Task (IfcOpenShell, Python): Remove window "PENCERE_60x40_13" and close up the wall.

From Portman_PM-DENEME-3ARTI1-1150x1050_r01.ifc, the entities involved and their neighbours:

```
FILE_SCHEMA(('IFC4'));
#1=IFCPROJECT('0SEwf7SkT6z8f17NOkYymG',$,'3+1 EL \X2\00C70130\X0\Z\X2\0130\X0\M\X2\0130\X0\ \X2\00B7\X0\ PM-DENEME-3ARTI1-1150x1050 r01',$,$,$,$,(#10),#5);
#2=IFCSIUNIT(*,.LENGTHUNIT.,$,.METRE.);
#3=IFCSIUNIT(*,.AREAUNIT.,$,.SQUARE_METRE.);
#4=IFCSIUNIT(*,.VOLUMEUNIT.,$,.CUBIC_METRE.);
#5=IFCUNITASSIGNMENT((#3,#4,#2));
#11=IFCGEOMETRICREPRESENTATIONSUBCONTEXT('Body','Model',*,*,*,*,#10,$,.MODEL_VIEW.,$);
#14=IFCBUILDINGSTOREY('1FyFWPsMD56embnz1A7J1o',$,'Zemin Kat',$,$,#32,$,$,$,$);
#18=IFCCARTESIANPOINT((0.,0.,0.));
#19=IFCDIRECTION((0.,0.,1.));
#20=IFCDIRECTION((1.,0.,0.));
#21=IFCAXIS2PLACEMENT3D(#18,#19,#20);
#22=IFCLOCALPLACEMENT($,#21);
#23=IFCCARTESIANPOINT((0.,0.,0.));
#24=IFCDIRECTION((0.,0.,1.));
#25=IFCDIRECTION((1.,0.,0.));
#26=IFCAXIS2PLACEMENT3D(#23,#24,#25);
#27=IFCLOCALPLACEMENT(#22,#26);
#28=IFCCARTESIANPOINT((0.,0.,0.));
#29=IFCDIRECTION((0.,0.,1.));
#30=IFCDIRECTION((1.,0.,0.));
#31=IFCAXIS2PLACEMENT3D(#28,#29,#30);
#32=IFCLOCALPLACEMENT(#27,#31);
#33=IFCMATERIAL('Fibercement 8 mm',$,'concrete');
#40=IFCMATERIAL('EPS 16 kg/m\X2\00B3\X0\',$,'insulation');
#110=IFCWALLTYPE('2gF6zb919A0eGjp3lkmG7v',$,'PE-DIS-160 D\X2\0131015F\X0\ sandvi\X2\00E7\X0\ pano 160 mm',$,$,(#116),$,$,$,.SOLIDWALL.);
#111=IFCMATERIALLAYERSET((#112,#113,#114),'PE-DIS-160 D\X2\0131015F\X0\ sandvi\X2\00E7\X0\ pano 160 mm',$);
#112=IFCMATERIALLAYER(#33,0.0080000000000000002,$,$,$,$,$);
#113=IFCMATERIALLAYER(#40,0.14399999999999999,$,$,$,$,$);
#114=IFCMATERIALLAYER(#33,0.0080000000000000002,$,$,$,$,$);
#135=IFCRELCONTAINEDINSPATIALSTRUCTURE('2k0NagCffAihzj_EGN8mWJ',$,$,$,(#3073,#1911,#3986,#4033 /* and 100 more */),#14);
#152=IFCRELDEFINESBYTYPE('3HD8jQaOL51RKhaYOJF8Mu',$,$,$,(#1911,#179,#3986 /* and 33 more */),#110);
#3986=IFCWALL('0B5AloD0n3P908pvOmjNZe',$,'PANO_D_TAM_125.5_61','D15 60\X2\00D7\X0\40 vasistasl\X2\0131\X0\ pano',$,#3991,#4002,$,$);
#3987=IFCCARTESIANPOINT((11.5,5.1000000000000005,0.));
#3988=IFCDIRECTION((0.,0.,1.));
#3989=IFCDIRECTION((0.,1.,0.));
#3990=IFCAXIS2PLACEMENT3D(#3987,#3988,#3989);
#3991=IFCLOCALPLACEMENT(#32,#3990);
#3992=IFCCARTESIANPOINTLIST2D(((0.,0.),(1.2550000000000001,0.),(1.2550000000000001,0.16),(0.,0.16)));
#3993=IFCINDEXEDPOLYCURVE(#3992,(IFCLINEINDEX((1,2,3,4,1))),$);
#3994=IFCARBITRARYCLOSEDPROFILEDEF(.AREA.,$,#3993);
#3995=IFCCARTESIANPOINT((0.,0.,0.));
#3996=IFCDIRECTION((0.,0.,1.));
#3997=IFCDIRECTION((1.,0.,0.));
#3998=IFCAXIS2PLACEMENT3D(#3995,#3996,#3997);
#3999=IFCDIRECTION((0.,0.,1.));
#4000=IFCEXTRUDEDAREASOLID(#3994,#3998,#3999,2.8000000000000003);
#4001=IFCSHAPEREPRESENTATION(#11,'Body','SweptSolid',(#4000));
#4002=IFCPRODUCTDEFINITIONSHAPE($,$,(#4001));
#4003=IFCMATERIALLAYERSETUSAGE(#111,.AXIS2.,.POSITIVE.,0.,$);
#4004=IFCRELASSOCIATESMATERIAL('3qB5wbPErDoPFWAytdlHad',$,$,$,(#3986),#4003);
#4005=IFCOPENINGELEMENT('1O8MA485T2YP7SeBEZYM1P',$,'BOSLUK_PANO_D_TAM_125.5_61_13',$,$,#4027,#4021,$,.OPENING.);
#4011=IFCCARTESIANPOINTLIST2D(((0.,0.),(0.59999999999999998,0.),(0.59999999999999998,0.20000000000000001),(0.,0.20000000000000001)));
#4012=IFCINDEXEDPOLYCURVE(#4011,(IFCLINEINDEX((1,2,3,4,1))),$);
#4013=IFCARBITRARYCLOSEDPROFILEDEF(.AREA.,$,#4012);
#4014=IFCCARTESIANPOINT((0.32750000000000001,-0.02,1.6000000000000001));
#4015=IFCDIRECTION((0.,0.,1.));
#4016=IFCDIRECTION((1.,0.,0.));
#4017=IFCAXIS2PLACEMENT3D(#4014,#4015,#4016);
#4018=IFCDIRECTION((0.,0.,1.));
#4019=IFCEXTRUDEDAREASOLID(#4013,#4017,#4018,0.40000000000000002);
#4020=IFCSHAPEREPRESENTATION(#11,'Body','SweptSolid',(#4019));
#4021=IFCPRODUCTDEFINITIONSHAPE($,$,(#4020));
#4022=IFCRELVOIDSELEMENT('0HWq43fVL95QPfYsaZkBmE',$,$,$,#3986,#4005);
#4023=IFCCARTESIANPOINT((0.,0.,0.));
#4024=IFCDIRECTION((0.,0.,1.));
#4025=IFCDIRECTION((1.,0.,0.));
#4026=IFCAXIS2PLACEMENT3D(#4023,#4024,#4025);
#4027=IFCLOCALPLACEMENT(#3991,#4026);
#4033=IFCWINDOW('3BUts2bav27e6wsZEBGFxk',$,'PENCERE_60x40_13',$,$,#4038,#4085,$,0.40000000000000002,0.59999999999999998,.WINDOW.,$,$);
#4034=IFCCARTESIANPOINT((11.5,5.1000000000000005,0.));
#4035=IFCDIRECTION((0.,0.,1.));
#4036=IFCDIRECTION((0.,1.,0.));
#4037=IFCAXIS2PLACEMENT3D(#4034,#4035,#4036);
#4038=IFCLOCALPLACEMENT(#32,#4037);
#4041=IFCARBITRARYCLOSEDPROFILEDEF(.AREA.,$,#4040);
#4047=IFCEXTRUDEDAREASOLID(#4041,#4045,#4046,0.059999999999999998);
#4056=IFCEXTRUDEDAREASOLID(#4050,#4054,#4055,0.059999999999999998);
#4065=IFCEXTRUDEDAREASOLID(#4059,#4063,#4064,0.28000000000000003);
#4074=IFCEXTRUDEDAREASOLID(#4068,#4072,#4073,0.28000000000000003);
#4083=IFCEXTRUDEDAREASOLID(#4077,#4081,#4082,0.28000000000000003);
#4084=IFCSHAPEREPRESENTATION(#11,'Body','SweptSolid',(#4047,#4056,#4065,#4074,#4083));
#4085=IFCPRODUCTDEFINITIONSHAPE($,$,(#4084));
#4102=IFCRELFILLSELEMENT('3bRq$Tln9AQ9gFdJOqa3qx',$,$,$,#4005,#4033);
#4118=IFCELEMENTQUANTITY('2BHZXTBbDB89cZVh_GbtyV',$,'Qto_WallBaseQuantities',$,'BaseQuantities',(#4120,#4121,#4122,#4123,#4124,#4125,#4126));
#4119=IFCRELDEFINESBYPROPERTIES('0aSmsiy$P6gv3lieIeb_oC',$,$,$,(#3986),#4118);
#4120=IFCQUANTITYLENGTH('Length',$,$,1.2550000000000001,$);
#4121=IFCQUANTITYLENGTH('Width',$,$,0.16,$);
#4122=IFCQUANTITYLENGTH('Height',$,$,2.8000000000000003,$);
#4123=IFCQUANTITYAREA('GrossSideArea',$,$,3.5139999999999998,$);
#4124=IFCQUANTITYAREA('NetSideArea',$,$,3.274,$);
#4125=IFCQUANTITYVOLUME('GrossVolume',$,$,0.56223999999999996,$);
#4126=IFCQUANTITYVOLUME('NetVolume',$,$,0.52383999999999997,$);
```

```python
import ifcopenshell
import ifcopenshell.api.feature
import ifcopenshell.api.pset
import ifcopenshell.api.root
import ifcopenshell.geom
import ifcopenshell.util.element
import ifcopenshell.util.shape
import ifcopenshell.util.unit

model = ifcopenshell.open("Portman_PM-DENEME-3ARTI1-1150x1050_r01.ifc")
area_scale = ifcopenshell.util.unit.calculate_unit_scale(model, "AREAUNIT")
volume_scale = ifcopenshell.util.unit.calculate_unit_scale(model, "VOLUMEUNIT")
settings = ifcopenshell.geom.settings()


def volume(element):
    """Net volume in cubic metres, openings subtracted."""
    shape = ifcopenshell.geom.create_shape(settings, element)
    return ifcopenshell.util.shape.get_volume(shape.geometry)


window = model.by_id(4033)
opening = window.FillsVoids[0].RelatingOpeningElement
wall = opening.VoidsElements[0].RelatingBuildingElement
before = volume(wall)

ifcopenshell.api.root.remove_product(model, product=window)
ifcopenshell.api.feature.remove_feature(model, feature=opening)

after = volume(wall)
thickness = 0.16  # wall thickness in metres

# Update the wall's stored quantities.
qto = model.by_id(ifcopenshell.util.element.get_pset(wall, "Qto_WallBaseQuantities", should_inherit=False)["id"])
ifcopenshell.api.pset.edit_qto(model, qto=qto, properties={
    "NetSideArea": after / thickness / area_scale,
    "NetVolume": after / volume_scale,
})

print(f"wall volume {before:.3f} -> {after:.3f} m3")

model.write("Portman_PM-DENEME-3ARTI1-1150x1050_r01_v2.ifc")
```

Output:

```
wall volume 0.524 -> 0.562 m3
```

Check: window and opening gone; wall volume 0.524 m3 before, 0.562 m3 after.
